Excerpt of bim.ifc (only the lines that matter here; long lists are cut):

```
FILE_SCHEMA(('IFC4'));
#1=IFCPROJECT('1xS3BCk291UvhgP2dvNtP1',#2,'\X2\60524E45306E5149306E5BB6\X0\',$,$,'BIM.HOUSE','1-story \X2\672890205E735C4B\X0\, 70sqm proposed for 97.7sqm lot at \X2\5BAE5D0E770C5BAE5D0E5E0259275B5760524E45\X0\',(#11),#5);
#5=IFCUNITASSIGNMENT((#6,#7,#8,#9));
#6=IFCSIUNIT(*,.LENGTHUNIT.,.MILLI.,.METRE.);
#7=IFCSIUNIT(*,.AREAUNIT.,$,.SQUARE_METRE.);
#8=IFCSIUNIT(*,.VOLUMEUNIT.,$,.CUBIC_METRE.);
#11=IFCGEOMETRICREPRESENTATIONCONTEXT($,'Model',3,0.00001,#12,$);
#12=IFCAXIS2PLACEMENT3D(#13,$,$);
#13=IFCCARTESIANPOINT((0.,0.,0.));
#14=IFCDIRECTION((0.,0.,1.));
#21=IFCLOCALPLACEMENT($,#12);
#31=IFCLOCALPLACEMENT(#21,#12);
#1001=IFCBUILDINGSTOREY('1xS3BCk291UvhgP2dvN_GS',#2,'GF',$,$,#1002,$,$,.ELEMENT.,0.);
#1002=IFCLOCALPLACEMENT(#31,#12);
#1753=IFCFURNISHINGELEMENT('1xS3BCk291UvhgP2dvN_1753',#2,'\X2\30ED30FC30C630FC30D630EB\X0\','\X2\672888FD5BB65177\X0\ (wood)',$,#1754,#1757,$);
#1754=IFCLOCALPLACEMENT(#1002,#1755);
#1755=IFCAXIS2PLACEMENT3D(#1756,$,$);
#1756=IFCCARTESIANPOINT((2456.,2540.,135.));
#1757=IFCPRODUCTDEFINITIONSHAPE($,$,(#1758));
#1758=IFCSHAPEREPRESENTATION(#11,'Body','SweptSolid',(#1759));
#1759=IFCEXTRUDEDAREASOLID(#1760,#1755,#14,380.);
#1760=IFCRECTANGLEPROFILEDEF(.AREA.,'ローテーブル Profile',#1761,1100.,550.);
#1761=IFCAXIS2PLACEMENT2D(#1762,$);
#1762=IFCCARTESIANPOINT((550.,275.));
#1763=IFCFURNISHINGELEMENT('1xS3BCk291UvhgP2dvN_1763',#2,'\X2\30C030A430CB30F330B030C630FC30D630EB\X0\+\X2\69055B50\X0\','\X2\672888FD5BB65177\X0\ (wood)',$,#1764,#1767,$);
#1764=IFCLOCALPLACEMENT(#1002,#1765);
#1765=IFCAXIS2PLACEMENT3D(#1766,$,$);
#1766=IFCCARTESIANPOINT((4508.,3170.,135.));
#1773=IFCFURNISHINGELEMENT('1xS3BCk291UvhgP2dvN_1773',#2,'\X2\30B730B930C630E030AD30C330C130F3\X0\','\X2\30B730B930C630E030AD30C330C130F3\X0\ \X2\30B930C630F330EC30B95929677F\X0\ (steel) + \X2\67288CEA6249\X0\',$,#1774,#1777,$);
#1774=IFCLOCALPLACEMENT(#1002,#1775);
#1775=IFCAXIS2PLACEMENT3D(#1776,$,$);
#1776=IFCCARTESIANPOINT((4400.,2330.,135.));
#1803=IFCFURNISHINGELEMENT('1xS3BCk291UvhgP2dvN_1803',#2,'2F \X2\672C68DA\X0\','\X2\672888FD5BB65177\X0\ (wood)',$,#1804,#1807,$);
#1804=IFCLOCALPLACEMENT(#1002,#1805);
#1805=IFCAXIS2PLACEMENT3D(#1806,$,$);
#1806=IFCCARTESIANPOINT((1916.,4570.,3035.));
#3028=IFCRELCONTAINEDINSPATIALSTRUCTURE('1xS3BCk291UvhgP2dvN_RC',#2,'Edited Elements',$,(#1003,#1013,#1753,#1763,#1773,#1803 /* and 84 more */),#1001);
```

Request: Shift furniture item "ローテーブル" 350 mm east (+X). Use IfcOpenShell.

```python
import ifcopenshell
import ifcopenshell.api.geometry
import ifcopenshell.util.placement

model = ifcopenshell.open("bim.ifc")

item = model.by_guid("1xS3BCk291UvhgP2dvN_1753")
matrix = ifcopenshell.util.placement.get_local_placement(item.ObjectPlacement)
matrix[0, 3] += 350.0
ifcopenshell.api.geometry.edit_object_placement(model, product=item, matrix=matrix, is_si=False)

print(ifcopenshell.util.placement.get_local_placement(item.ObjectPlacement).round(3) + 0.0)

model.write("bim_v2.ifc")
```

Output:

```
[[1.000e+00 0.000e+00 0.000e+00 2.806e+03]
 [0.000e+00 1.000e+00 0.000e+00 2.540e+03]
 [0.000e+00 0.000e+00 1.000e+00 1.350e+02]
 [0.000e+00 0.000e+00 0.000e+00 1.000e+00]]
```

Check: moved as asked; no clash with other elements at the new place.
